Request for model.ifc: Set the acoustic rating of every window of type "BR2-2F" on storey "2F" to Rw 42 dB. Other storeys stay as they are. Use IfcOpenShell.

First a look at what the model holds.

```python
import ifcopenshell
import ifcopenshell.util.element

model = ifcopenshell.open("model.ifc")
print(model.schema)
storey = next(s for s in model.by_type("IfcBuildingStorey") if s.Name == "2F")
windows = [e for e in ifcopenshell.util.element.get_decomposition(storey) if e.is_a("IfcWindow")]
seen = {}
for e in windows:
    element_type = ifcopenshell.util.element.get_type(e)
    key = (element_type.Name if element_type != e and element_type else None, ifcopenshell.util.element.get_pset(e, "Pset_WindowCommon", "AcousticRating"))
    seen[key] = seen.get(key, 0) + 1
for (name, value), count in sorted(seen.items(), key=str):
    print(count, "x", name, "|", value)
```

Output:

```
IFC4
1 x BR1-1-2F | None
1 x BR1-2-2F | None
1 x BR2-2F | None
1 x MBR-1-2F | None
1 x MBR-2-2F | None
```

```python
import ifcopenshell
import ifcopenshell.api.pset
import ifcopenshell.util.element

model = ifcopenshell.open("model.ifc")

storey = next(s for s in model.by_type("IfcBuildingStorey") if s.Name == "2F")
windows = [e for e in ifcopenshell.util.element.get_decomposition(storey) if e.is_a("IfcWindow")]

count = 0
for e in windows:
    element_type = ifcopenshell.util.element.get_type(e)
    if element_type in (None, e) or element_type.Name != "BR2-2F":
        continue
    # add_pset returns the element's existing set when there is one.
    pset = ifcopenshell.api.pset.add_pset(model, product=e, name="Pset_WindowCommon")
    ifcopenshell.api.pset.edit_pset(model, pset=pset, properties={"AcousticRating": "Rw 42 dB"})
    count += 1

print(count, "windows updated")

model.write("model_edited.ifc")
```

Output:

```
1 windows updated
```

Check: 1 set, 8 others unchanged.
